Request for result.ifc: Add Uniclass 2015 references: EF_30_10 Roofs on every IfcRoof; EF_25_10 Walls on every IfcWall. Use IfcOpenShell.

First a look at what the model holds.

```python
import ifcopenshell

model = ifcopenshell.open("result.ifc")
print(model.schema)
print("classifications:", [c.Name for c in model.by_type("IfcClassification")])
for ifc_class in ("IfcDoor", "IfcRoof", "IfcStair", "IfcWall", "IfcWindow"):
    print(ifc_class, len(model.by_type(ifc_class)))
```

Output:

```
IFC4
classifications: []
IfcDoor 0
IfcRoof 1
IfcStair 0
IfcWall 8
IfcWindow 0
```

```python
import ifcopenshell
import ifcopenshell.api.classification

model = ifcopenshell.open("result.ifc")

system = ifcopenshell.api.classification.add_classification(model, classification="Uniclass 2015")

codes = {
    "IfcRoof": ("EF_30_10", "Roofs"),
    "IfcWall": ("EF_25_10", "Walls"),
}
for ifc_class, (code, name) in codes.items():
    products = model.by_type(ifc_class)
    ifcopenshell.api.classification.add_reference(
        model, products=products, classification=system, identification=code, name=name
    )
    print(code, len(products))

model.write("result_updated.ifc")
```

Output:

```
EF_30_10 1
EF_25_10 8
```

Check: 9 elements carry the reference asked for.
